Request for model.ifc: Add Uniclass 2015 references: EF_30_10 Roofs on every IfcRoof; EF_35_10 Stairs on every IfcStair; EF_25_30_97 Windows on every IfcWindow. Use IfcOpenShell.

First a look at what the model holds.

```python
import ifcopenshell

model = ifcopenshell.open("model.ifc")
print(model.schema)
print("classifications:", [c.Name for c in model.by_type("IfcClassification")])
for ifc_class in ("IfcDoor", "IfcRoof", "IfcStair", "IfcWall", "IfcWindow"):
    print(ifc_class, len(model.by_type(ifc_class)))
```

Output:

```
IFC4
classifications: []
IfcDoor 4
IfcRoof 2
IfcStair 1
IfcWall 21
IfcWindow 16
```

```python
import ifcopenshell
import ifcopenshell.api.classification

model = ifcopenshell.open("model.ifc")

system = ifcopenshell.api.classification.add_classification(model, classification="Uniclass 2015")

codes = {
    "IfcRoof": ("EF_30_10", "Roofs"),
    "IfcStair": ("EF_35_10", "Stairs"),
    "IfcWindow": ("EF_25_30_97", "Windows"),
}
for ifc_class, (code, name) in codes.items():
    products = model.by_type(ifc_class)
    ifcopenshell.api.classification.add_reference(
        model, products=products, classification=system, identification=code, name=name
    )
    print(code, len(products))

model.write("model-out.ifc")
```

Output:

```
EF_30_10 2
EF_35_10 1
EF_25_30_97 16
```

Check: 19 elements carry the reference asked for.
